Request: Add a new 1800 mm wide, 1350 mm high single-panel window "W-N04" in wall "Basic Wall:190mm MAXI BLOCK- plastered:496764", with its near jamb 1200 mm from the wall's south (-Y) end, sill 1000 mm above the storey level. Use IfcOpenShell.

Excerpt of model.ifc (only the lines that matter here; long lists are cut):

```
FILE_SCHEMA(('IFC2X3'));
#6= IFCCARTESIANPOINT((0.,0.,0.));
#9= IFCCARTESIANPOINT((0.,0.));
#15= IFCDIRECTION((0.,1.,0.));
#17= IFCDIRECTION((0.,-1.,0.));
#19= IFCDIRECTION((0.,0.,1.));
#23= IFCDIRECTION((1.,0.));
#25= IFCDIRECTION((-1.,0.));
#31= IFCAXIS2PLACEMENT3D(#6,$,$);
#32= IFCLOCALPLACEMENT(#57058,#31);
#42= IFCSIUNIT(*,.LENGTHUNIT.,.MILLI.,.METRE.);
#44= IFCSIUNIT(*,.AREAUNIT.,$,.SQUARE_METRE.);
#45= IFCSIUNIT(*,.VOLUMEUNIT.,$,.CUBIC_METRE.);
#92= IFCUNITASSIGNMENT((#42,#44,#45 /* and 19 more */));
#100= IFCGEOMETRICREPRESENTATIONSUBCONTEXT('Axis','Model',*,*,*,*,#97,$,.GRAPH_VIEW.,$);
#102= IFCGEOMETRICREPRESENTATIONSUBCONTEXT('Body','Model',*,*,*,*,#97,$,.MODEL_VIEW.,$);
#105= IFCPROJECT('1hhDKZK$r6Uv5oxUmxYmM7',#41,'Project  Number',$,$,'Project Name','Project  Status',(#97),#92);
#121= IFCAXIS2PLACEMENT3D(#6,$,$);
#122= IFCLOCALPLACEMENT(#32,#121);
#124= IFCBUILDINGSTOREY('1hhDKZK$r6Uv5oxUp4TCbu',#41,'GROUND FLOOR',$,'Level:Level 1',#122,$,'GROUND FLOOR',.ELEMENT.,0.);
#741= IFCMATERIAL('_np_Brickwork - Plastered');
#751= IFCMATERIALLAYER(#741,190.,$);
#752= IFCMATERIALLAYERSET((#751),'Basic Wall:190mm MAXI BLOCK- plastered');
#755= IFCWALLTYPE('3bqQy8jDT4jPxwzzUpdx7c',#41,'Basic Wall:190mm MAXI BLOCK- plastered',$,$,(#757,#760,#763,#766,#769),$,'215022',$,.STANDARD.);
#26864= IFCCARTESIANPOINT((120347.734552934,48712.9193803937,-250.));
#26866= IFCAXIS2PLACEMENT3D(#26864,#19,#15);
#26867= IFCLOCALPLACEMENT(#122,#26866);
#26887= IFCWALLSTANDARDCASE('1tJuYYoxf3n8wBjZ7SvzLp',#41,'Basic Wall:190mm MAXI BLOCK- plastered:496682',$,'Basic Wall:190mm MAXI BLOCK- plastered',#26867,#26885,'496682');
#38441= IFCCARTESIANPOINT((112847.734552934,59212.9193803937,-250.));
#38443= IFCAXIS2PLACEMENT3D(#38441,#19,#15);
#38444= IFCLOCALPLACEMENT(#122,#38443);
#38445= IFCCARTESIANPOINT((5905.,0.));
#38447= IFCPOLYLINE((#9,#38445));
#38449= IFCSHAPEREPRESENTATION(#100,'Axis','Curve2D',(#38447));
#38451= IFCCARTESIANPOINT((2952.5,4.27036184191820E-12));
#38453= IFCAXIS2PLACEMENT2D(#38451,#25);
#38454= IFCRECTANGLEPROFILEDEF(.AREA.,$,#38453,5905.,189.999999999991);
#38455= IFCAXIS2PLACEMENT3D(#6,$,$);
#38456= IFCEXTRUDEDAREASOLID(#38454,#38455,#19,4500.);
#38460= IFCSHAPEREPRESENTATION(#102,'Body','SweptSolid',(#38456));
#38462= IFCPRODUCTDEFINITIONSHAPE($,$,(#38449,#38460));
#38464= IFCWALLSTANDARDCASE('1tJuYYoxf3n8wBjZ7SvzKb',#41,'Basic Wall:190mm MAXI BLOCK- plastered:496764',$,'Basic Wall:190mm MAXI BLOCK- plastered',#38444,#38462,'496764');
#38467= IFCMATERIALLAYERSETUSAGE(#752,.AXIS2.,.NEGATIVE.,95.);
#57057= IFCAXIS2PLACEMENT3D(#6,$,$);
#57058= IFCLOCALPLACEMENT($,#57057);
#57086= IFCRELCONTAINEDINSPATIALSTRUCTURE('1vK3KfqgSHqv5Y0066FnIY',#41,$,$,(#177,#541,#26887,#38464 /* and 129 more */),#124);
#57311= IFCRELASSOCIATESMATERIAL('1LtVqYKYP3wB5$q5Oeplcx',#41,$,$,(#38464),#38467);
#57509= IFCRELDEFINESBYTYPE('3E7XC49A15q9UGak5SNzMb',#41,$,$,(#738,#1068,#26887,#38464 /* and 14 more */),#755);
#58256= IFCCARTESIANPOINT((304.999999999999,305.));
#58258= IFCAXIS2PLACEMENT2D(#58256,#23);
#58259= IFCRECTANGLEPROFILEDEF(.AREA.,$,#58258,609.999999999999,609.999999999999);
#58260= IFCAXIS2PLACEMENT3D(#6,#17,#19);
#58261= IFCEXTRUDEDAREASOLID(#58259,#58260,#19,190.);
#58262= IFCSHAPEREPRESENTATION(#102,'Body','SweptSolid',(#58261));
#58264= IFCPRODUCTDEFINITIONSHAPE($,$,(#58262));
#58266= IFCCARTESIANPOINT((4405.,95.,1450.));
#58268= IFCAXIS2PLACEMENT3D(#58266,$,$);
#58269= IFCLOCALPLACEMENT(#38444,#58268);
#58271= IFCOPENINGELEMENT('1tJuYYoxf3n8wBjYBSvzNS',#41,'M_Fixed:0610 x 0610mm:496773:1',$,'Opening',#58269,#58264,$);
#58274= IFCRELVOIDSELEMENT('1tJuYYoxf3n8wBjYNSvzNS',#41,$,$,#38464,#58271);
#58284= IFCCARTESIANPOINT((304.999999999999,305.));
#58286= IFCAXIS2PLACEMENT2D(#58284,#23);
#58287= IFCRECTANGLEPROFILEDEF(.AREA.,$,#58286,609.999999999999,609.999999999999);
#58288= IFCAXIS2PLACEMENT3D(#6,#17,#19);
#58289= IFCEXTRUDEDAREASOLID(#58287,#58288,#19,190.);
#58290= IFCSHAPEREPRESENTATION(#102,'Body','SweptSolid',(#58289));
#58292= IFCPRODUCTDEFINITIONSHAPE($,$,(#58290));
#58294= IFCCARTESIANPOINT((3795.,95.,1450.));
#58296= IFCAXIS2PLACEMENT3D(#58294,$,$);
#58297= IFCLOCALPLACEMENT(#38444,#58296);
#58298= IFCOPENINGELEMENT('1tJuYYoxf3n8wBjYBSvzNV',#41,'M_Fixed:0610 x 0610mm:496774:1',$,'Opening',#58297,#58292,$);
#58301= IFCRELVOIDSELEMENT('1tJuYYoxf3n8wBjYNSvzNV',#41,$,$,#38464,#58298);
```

```python
import numpy as np
import ifcopenshell
import ifcopenshell.api.feature
import ifcopenshell.api.geometry
import ifcopenshell.api.root
import ifcopenshell.api.spatial
import ifcopenshell.api.type
import ifcopenshell.geom
import ifcopenshell.util.element
import ifcopenshell.util.placement
import ifcopenshell.util.representation
import ifcopenshell.util.shape
import ifcopenshell.util.unit

model = ifcopenshell.open("model.ifc")
unit_scale = ifcopenshell.util.unit.calculate_unit_scale(model)
settings = ifcopenshell.geom.settings()


def volume(element):
    """Net volume in cubic metres, openings subtracted."""
    shape = ifcopenshell.geom.create_shape(settings, element)
    return ifcopenshell.util.shape.get_volume(shape.geometry)


wall = model.by_guid("1tJuYYoxf3n8wBjZ7SvzKb")
storey = ifcopenshell.util.element.get_container(wall, ifc_class="IfcBuildingStorey")
context = ifcopenshell.util.representation.get_context(model, "Model", "Body", "MODEL_VIEW")
before = volume(wall)

width, height, from_end, sill = 1.8, 1.35, 1.2, 1  # metres

# The wall runs along its own X axis, and the end named is its -X end.
wall_shape = ifcopenshell.geom.create_shape(settings, wall)
x, y, z = ifcopenshell.util.shape.get_vertices(wall_shape.geometry).T
start = x.min() + from_end
face, thickness = float(y.min()), float(y.max() - y.min())
wall_matrix = ifcopenshell.util.placement.get_local_placement(wall.ObjectPlacement)
level = ifcopenshell.util.placement.get_local_placement(storey.ObjectPlacement)[2, 3]


def in_wall(x, y):
    """Placement at x, y metres in the wall's axes, at sill height."""
    matrix = wall_matrix.copy()
    matrix[:, 3] = wall_matrix @ np.array([x / unit_scale, y / unit_scale, 0.0, 1.0])
    matrix[2, 3] = level + sill / unit_scale
    return matrix


# Opening: a box that overshoots both wall faces by 50 mm.
opening = ifcopenshell.api.root.create_entity(model, ifc_class="IfcOpeningElement")
box = ifcopenshell.api.geometry.add_wall_representation(
    model, context=context, length=width, height=height, thickness=thickness + 0.1
)
ifcopenshell.api.geometry.assign_representation(model, product=opening, representation=box)
ifcopenshell.api.geometry.edit_object_placement(model, product=opening, matrix=in_wall(start, face - 0.05), is_si=False)
ifcopenshell.api.feature.add_feature(model, feature=opening, element=wall)

window = ifcopenshell.api.root.create_entity(model, ifc_class="IfcWindow", name="W-N04")
window.OverallWidth, window.OverallHeight = width / unit_scale, height / unit_scale
body = ifcopenshell.api.geometry.add_window_representation(
    model,
    context=context,
    overall_width=window.OverallWidth,
    overall_height=window.OverallHeight,
    partition_type="SINGLE_PANEL",
)
ifcopenshell.api.geometry.assign_representation(model, product=window, representation=body)
ifcopenshell.api.spatial.assign_container(model, products=[window], relating_structure=storey)
fills = ifcopenshell.api.feature.add_filling(model, opening=opening, element=window)
fills.OwnerHistory = window.OwnerHistory  # required in IFC2X3

# IFC2X3 keeps the operation on the window style.
style = ifcopenshell.api.root.create_entity(model, ifc_class="IfcWindowStyle", name="W-N04")
style.OperationType, style.ConstructionType = "SINGLE_PANEL", "NOTDEFINED"
style.ParameterTakesPrecedence = style.Sizeable = False
ifcopenshell.api.type.assign_type(model, related_objects=[window], relating_type=style)

# Centre the window in the wall's thickness.
ifcopenshell.api.geometry.edit_object_placement(model, product=window, matrix=in_wall(start, face), is_si=False)
window_shape = ifcopenshell.geom.create_shape(settings, window)
depth = ifcopenshell.util.shape.get_vertices(window_shape.geometry)[:, 1]
offset = face + thickness / 2 - (depth.min() + depth.max()) / 2
ifcopenshell.api.geometry.edit_object_placement(model, product=window, matrix=in_wall(start, offset), is_si=False)

after = volume(wall)

print(f"wall volume {before:.3f} -> {after:.3f} m3")

model.write("model_updated.ifc")
```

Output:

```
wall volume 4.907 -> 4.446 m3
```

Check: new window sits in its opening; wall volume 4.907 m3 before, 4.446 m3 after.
